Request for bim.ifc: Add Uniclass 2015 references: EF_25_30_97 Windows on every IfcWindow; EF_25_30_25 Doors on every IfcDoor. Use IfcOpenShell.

First a look at what the model holds.

```python
import ifcopenshell

model = ifcopenshell.open("bim.ifc")
print(model.schema)
print("classifications:", [c.Name for c in model.by_type("IfcClassification")])
for ifc_class in ("IfcDoor", "IfcRoof", "IfcStair", "IfcWall", "IfcWindow"):
    print(ifc_class, len(model.by_type(ifc_class)))
```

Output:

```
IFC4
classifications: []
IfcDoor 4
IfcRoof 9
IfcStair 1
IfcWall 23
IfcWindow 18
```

```python
import ifcopenshell
import ifcopenshell.api.classification

model = ifcopenshell.open("bim.ifc")

system = ifcopenshell.api.classification.add_classification(model, classification="Uniclass 2015")

codes = {
    "IfcWindow": ("EF_25_30_97", "Windows"),
    "IfcDoor": ("EF_25_30_25", "Doors"),
}
for ifc_class, (code, name) in codes.items():
    products = model.by_type(ifc_class)
    ifcopenshell.api.classification.add_reference(
        model, products=products, classification=system, identification=code, name=name
    )
    print(code, len(products))

model.write("bim_rev.ifc")
```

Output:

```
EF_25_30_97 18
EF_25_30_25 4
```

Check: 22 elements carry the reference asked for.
